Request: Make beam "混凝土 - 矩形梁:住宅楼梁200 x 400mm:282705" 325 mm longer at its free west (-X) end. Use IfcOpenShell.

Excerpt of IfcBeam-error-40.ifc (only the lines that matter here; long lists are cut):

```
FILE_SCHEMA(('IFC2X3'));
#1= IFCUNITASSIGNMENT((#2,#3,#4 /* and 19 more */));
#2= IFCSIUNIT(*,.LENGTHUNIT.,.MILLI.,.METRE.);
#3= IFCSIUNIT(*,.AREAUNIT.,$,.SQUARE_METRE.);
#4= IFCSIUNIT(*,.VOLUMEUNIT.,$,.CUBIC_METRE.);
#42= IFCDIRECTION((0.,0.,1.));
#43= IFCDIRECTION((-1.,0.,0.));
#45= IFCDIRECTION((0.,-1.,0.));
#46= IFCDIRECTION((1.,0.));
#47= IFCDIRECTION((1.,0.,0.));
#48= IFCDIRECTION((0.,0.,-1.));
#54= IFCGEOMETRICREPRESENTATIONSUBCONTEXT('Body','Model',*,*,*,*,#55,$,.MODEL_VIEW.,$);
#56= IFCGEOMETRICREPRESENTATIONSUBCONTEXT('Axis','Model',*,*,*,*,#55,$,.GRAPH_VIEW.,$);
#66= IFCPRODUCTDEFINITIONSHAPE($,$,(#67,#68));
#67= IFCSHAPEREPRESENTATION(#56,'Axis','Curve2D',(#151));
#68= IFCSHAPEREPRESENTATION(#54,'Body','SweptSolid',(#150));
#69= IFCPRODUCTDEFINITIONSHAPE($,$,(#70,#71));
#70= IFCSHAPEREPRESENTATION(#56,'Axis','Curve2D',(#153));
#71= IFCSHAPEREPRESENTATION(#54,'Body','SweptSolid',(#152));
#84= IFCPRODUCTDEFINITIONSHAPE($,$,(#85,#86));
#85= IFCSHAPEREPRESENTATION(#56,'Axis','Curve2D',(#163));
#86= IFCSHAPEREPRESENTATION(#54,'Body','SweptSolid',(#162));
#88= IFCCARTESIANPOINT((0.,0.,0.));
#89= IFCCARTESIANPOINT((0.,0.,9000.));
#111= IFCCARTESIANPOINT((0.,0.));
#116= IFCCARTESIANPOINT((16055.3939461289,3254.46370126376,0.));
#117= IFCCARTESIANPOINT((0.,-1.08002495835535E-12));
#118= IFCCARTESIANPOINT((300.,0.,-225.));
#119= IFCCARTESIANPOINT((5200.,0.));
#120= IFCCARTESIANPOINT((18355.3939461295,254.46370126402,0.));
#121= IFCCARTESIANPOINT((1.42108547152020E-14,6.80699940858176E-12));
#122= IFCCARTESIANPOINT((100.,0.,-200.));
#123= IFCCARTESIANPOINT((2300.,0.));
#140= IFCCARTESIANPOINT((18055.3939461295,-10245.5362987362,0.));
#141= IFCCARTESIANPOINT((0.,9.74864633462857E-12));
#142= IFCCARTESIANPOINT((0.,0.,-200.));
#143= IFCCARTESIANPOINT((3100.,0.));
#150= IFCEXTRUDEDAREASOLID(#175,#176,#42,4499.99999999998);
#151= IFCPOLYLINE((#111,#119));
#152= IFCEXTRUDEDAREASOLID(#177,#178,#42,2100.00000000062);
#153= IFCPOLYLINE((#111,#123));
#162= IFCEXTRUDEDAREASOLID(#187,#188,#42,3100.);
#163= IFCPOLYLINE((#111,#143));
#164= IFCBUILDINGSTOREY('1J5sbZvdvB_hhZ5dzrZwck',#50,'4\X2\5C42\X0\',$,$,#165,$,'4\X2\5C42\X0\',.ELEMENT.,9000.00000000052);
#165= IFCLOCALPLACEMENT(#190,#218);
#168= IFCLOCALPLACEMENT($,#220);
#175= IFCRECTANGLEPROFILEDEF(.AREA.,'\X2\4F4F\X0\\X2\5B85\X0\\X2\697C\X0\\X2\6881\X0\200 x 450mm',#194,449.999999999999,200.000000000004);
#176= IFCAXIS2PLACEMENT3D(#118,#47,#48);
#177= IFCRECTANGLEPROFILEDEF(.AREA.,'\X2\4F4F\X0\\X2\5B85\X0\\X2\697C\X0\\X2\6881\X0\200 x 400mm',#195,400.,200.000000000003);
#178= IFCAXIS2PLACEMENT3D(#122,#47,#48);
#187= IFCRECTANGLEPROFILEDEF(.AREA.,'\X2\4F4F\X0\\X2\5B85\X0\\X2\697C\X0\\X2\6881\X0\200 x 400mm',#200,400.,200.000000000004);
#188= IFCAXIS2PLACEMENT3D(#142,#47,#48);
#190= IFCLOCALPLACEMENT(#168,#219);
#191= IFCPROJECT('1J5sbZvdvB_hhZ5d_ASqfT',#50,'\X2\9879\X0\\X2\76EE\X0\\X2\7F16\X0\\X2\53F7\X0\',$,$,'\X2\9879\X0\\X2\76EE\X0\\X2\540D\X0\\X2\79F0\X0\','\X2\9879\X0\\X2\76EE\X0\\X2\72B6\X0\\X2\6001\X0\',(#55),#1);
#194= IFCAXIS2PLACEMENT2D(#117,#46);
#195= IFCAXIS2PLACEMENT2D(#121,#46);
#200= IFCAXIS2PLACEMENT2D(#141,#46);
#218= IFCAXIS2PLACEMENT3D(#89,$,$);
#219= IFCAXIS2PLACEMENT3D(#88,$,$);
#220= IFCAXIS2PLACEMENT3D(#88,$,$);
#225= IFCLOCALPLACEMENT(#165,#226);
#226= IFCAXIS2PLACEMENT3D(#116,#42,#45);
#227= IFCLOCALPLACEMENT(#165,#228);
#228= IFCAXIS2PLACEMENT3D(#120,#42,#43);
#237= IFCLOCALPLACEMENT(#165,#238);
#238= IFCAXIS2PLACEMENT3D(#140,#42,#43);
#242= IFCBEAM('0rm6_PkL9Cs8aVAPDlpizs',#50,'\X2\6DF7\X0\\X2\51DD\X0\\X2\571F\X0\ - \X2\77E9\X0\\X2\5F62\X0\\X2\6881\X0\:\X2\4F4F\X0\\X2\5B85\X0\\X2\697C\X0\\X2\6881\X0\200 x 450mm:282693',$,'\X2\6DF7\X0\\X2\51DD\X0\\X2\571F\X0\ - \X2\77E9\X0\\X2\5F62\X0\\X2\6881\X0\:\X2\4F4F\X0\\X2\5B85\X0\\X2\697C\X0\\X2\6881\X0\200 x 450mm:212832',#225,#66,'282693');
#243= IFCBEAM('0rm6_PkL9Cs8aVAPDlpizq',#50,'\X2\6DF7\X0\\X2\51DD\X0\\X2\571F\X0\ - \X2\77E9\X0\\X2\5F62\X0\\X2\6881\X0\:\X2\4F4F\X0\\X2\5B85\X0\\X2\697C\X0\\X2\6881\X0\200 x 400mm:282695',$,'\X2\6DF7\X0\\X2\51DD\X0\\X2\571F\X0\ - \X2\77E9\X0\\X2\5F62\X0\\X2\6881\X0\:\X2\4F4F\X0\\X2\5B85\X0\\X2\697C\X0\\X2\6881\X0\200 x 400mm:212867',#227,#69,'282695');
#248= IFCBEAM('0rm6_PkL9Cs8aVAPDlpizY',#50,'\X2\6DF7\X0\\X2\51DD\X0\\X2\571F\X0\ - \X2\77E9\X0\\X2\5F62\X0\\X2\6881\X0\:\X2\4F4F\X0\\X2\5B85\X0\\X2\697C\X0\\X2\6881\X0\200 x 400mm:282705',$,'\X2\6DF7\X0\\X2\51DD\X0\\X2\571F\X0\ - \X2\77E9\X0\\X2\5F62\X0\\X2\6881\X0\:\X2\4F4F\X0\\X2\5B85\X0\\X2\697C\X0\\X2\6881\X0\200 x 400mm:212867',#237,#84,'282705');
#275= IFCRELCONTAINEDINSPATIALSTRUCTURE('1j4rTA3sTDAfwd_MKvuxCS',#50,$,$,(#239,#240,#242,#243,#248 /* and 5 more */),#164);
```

```python
import numpy as np
import ifcopenshell
import ifcopenshell.util.representation

model = ifcopenshell.open("IfcBeam-error-40.ifc")

member = model.by_guid("0rm6_PkL9Cs8aVAPDlpizY")
change = 325.0

# The extrusion runs towards the end named, so only its depth changes.
body = ifcopenshell.util.representation.get_representation(member, "Model", "Body")
solid = body.Items[0]
old_length = solid.Depth
solid.Depth += change

# Move the axis end point with it.
axis = next(r for r in member.Representation.Representations if r.RepresentationIdentifier == "Axis").Items[0]
start, end = (np.array(p.Coordinates) for p in axis.Points)
end = end + (end - start) / np.linalg.norm(end - start) * change
point = model.createIfcCartesianPoint(end.tolist())
axis.Points = [axis.Points[0], point]

print(f"length {old_length:g} -> {solid.Depth:g}")

model.write("IfcBeam-error-40_edited.ifc")
```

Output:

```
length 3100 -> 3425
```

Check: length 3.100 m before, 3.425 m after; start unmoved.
